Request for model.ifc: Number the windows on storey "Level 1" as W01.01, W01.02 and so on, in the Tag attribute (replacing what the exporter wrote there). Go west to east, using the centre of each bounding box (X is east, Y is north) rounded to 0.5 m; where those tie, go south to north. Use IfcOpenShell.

First a look at what the model holds.

```python
import ifcopenshell
import ifcopenshell.util.element
import ifcopenshell.util.placement

model = ifcopenshell.open("model.ifc")
print(model.schema)
storey = next(s for s in model.by_type("IfcBuildingStorey") if s.Name == "Level 1")
windows = [e for e in ifcopenshell.util.element.get_decomposition(storey) if e.is_a("IfcWindow")]
for e in sorted(windows, key=lambda e: e.id()):
    origin = ifcopenshell.util.placement.get_local_placement(e.ObjectPlacement)[:3, 3]
    print(e.id(), e.Tag, e.Name, origin.round(2) + 0.0, sep=" | ")
```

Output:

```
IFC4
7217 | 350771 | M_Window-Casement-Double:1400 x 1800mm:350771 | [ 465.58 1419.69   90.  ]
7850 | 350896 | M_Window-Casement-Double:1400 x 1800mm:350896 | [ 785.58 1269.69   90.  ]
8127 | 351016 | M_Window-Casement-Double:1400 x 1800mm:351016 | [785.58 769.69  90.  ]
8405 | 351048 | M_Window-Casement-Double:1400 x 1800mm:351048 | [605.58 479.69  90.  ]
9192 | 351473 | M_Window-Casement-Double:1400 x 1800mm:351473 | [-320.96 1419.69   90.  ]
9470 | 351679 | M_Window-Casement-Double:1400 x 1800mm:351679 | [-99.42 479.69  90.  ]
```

```python
import ifcopenshell
import ifcopenshell.geom
import ifcopenshell.util.element
import ifcopenshell.util.shape

model = ifcopenshell.open("model.ifc")
settings = ifcopenshell.geom.settings()
settings.set("use-world-coords", True)


def centre(element):
    shape = ifcopenshell.geom.create_shape(settings, element)
    return ifcopenshell.util.shape.get_bbox_centroid(shape.geometry)


storey = next(s for s in model.by_type("IfcBuildingStorey") if s.Name == "Level 1")
windows = [e for e in ifcopenshell.util.element.get_decomposition(storey) if e.is_a("IfcWindow")]

# Insertion points can sit at a corner or the storey origin, so sort by the geometry (in metres).
centres = {e: centre(e) for e in windows}
windows.sort(key=lambda e: (round(centres[e][0] / 0.5), centres[e][1]))

for i, e in enumerate(windows, start=1):
    number = f"W01.{i:02d}"
    e.Tag = number
    print(e.id(), number)

model.write("model-out.ifc")
```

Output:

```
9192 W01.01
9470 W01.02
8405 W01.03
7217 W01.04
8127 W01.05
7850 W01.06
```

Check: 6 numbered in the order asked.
